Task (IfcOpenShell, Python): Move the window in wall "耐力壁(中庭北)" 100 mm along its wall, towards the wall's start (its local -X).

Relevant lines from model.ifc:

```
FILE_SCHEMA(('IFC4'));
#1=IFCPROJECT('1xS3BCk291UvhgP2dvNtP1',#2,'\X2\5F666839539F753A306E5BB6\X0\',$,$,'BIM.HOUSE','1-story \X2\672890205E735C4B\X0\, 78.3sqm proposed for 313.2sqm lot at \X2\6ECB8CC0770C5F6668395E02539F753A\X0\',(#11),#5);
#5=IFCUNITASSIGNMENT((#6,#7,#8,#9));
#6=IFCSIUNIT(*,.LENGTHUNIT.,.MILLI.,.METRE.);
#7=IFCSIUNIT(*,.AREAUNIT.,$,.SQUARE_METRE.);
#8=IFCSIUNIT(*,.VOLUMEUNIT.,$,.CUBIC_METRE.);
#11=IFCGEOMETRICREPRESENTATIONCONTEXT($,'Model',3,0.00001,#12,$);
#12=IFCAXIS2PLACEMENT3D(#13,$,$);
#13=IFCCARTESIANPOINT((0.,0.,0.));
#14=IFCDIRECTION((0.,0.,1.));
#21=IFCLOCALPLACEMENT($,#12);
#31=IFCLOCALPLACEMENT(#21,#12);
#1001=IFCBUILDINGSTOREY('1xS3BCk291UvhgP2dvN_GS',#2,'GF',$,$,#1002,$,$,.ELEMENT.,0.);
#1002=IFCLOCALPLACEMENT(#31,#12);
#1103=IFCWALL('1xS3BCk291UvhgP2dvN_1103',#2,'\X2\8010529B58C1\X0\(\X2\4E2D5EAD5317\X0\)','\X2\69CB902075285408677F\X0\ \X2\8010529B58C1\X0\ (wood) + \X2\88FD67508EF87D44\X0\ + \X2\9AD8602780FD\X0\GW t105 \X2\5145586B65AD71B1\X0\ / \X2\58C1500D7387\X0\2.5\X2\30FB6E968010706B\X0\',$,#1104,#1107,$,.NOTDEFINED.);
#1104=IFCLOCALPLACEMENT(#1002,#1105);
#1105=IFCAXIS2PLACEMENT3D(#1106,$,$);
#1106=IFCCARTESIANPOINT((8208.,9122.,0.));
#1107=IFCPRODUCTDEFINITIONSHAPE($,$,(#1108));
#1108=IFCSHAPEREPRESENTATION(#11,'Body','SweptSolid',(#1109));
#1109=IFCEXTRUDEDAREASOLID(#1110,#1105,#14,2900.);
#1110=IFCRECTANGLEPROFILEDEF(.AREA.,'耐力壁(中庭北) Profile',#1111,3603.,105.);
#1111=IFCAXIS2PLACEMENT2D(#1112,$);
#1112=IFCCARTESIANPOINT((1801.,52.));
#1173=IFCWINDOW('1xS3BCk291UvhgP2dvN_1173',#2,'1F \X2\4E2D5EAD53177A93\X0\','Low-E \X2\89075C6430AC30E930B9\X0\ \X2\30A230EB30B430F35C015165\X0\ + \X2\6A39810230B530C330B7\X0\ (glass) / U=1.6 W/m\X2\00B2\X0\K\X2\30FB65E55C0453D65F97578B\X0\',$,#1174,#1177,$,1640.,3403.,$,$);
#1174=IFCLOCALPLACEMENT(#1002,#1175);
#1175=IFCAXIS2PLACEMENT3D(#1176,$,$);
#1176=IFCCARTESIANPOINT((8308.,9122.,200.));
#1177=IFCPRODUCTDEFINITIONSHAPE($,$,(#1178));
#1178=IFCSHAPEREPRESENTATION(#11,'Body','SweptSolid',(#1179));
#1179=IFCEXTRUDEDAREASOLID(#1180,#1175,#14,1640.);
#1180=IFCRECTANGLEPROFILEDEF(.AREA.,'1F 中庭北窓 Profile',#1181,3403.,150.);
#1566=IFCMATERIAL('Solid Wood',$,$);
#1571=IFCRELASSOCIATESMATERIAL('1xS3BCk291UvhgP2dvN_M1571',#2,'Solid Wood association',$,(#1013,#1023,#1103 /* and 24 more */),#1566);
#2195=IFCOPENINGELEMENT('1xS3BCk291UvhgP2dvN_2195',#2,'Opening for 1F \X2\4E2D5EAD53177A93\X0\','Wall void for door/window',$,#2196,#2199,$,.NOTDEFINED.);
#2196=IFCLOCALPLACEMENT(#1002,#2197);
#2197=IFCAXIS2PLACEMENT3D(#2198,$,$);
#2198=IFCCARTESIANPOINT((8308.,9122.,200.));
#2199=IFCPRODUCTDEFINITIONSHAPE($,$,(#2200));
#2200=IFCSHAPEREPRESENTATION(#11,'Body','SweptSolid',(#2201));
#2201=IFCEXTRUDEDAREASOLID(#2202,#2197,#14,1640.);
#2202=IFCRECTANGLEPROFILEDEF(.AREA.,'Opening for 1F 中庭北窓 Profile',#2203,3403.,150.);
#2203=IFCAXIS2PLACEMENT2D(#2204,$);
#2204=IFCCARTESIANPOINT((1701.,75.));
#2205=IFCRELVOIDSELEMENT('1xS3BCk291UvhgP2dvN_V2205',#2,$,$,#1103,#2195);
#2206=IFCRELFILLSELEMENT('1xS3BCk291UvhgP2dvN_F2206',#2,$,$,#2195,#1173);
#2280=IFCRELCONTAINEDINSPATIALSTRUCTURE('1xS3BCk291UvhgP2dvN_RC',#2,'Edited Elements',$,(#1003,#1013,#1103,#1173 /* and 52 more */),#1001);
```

```python
import ifcopenshell
import ifcopenshell.api.geometry
import ifcopenshell.util.placement

model = ifcopenshell.open("model.ifc")

window = model.by_guid("1xS3BCk291UvhgP2dvN_1173")
opening = window.FillsVoids[0].RelatingOpeningElement
wall = opening.VoidsElements[0].RelatingBuildingElement

wall_matrix = ifcopenshell.util.placement.get_local_placement(wall.ObjectPlacement)
shift = wall_matrix[:3, 0] * -100.0
before = ifcopenshell.util.placement.get_local_placement(window.ObjectPlacement)[:3, 3].copy()

# The window is not placed relative to its opening, so move both.
for product in (opening, window):
    matrix = ifcopenshell.util.placement.get_local_placement(product.ObjectPlacement)
    matrix[:3, 3] += shift
    ifcopenshell.api.geometry.edit_object_placement(model, product=product, matrix=matrix, is_si=False)

after = ifcopenshell.util.placement.get_local_placement(window.ObjectPlacement)[:3, 3]
print("window moved by", (after - before).round(3) + 0.0)

model.write("model-out.ifc")
```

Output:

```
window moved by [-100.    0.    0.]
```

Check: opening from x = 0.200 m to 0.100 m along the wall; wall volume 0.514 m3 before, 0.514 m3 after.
